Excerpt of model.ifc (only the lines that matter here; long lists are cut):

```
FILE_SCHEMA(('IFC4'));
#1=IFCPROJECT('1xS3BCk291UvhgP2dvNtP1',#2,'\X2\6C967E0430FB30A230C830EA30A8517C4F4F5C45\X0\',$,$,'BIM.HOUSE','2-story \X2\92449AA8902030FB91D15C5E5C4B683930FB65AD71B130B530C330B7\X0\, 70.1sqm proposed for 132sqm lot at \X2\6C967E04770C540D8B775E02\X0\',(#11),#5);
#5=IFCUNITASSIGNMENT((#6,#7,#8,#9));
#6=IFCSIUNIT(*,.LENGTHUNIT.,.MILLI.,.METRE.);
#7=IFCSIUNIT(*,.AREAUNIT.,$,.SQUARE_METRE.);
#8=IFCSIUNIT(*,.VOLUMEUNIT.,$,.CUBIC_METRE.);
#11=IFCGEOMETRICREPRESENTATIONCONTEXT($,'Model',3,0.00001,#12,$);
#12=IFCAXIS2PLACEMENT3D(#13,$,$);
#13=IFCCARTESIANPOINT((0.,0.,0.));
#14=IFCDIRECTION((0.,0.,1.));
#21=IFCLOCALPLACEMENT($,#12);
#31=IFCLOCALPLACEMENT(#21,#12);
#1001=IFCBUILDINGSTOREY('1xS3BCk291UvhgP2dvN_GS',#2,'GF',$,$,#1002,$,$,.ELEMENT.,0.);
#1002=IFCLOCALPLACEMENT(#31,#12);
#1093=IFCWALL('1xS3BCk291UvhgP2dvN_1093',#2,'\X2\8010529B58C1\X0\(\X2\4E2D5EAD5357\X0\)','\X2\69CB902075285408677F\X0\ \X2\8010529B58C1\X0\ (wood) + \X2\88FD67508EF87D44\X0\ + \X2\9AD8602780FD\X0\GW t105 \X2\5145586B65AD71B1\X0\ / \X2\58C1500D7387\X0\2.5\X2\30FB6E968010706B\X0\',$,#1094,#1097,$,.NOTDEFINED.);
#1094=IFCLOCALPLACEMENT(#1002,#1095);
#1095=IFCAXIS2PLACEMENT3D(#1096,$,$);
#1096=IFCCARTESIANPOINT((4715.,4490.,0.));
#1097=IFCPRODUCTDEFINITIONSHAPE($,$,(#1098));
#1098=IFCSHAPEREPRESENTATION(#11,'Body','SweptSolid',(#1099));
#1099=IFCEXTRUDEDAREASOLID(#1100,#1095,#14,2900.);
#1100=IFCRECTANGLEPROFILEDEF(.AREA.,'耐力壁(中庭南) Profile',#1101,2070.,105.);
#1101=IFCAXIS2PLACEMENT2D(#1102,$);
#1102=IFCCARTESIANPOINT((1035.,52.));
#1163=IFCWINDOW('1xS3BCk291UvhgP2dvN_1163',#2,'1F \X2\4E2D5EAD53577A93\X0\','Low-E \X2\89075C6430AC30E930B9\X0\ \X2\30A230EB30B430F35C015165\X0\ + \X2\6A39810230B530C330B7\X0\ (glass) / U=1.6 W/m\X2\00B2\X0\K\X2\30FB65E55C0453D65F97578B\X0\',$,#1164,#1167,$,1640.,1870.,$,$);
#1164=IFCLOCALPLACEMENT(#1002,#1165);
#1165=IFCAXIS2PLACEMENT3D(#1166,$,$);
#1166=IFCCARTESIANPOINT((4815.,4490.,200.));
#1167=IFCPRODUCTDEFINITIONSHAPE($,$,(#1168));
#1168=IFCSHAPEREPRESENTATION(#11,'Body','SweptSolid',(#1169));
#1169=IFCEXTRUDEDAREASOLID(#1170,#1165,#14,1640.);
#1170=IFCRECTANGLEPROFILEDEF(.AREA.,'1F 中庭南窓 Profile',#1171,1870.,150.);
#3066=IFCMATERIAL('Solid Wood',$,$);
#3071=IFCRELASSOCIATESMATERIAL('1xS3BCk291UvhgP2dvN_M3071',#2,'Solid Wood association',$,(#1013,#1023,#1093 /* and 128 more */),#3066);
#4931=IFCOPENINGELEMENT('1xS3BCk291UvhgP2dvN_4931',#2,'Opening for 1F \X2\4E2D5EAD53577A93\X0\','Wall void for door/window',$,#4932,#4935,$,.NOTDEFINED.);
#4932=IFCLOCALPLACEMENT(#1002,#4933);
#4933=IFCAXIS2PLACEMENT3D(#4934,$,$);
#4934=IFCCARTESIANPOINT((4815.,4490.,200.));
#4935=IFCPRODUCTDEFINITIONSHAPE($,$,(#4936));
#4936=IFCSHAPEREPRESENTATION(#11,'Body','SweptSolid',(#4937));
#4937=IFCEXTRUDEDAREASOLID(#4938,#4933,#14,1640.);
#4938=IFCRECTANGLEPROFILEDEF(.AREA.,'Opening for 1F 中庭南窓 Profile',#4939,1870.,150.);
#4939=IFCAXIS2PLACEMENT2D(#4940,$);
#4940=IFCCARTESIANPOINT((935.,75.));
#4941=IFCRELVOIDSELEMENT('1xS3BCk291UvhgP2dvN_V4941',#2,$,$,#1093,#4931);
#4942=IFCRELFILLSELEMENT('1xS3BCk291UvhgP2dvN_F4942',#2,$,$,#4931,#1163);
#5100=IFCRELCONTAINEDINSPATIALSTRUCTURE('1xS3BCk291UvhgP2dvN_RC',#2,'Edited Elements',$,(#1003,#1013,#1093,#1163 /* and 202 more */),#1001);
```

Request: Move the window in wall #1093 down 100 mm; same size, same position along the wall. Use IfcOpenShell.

```python
import numpy as np
import ifcopenshell
import ifcopenshell.api.geometry
import ifcopenshell.util.placement
import ifcopenshell.util.unit

model = ifcopenshell.open("model.ifc")
unit_scale = ifcopenshell.util.unit.calculate_unit_scale(model)

window = model.by_guid("1xS3BCk291UvhgP2dvN_1163")
opening = window.FillsVoids[0].RelatingOpeningElement
dz = -0.1 / unit_scale

shift = np.array([0.0, 0.0, dz])
# The window is not placed relative to its opening, so move both.
for product in (opening, window):
    matrix = ifcopenshell.util.placement.get_local_placement(product.ObjectPlacement)
    matrix[:3, 3] += shift
    ifcopenshell.api.geometry.edit_object_placement(model, product=product, matrix=matrix, is_si=False)

print(f"moved by {dz * unit_scale:+.3f} m")

model.write("model-out.ifc")
```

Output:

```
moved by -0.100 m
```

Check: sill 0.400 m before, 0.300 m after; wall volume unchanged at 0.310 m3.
